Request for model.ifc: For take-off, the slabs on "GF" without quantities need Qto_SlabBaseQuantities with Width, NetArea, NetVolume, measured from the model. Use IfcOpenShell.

First a look at what the model holds.

```python
import ifcopenshell
import ifcopenshell.util.element
import ifcopenshell.util.unit

model = ifcopenshell.open("model.ifc")
print(model.schema)
for unit_type in ("LENGTHUNIT", "AREAUNIT", "VOLUMEUNIT"):
    print(unit_type, ifcopenshell.util.unit.calculate_unit_scale(model, unit_type))
storey = next(s for s in model.by_type("IfcBuildingStorey") if s.Name == "GF")
slabs = [e for e in ifcopenshell.util.element.get_decomposition(storey) if e.is_a("IfcSlab")]
for e in sorted(slabs, key=lambda e: e.id()):
    print(e.id(), e.is_a(), e.Name, list(ifcopenshell.util.element.get_psets(e, qtos_only=True)), sep=" | ")
```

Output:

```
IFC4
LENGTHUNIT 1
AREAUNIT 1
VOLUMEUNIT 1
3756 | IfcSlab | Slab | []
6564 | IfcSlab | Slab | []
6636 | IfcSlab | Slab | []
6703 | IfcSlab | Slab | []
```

```python
import ifcopenshell
import ifcopenshell.api.pset
import ifcopenshell.geom
import ifcopenshell.util.element
import ifcopenshell.util.shape
import ifcopenshell.util.unit

model = ifcopenshell.open("model.ifc")
unit_scale = ifcopenshell.util.unit.calculate_unit_scale(model)
area_scale = ifcopenshell.util.unit.calculate_unit_scale(model, "AREAUNIT")
volume_scale = ifcopenshell.util.unit.calculate_unit_scale(model, "VOLUMEUNIT")
settings = ifcopenshell.geom.settings()

storey = next(s for s in model.by_type("IfcBuildingStorey") if s.Name == "GF")
slabs = [e for e in ifcopenshell.util.element.get_decomposition(storey) if e.is_a("IfcSlab")]

for e in sorted(slabs, key=lambda e: e.id()):
    if ifcopenshell.util.element.get_psets(e, qtos_only=True, should_inherit=False):
        continue
    # Geometry comes back in metres, in the element's own axes.
    shape = ifcopenshell.geom.create_shape(settings, e)
    values = {
        "Width": ifcopenshell.util.shape.get_z(shape.geometry) / unit_scale,
        "NetArea": ifcopenshell.util.shape.get_footprint_area(shape.geometry) / area_scale,
        "NetVolume": ifcopenshell.util.shape.get_volume(shape.geometry) / volume_scale,
    }
    qto = ifcopenshell.api.pset.add_qto(model, product=e, name="Qto_SlabBaseQuantities")
    ifcopenshell.api.pset.edit_qto(model, qto=qto, properties=values)
    print(e.id(), {k: round(v, 3) for k, v in values.items()})

model.write("model_v2.ifc")
```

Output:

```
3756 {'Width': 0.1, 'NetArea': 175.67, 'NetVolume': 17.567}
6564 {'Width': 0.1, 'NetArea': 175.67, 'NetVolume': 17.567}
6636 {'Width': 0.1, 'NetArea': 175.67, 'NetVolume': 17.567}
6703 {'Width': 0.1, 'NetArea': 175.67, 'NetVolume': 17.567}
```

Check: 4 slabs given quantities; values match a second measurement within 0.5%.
